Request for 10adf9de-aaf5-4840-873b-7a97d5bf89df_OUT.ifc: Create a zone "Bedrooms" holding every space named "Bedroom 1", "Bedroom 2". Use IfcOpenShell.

First a look at what the model holds.

```python
import ifcopenshell

model = ifcopenshell.open("10adf9de-aaf5-4840-873b-7a97d5bf89df_OUT.ifc")
print(model.schema)
seen = {}
for space in model.by_type("IfcSpace"):
    seen[space.LongName] = seen.get(space.LongName, 0) + 1
for name, count in sorted(seen.items(), key=str):
    print(count, "x", name)
print("zones:", [z.Name for z in model.by_type("IfcZone")][:20])
```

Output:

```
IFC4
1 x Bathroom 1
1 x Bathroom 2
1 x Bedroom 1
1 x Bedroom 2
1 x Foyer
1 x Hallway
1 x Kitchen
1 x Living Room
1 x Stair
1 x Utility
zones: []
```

```python
import ifcopenshell
import ifcopenshell.api.group
import ifcopenshell.api.root

model = ifcopenshell.open("10adf9de-aaf5-4840-873b-7a97d5bf89df_OUT.ifc")

names = {"Bedroom 1", "Bedroom 2"}
spaces = [s for s in model.by_type("IfcSpace") if s.LongName in names]

zone = ifcopenshell.api.root.create_entity(model, ifc_class="IfcZone", name="Bedrooms")
ifcopenshell.api.group.assign_group(model, products=spaces, group=zone)
print(len(spaces), "spaces in", zone.Name)

model.write("10adf9de-aaf5-4840-873b-7a97d5bf89df_OUT_edited.ifc")
```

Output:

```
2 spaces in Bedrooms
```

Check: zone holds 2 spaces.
